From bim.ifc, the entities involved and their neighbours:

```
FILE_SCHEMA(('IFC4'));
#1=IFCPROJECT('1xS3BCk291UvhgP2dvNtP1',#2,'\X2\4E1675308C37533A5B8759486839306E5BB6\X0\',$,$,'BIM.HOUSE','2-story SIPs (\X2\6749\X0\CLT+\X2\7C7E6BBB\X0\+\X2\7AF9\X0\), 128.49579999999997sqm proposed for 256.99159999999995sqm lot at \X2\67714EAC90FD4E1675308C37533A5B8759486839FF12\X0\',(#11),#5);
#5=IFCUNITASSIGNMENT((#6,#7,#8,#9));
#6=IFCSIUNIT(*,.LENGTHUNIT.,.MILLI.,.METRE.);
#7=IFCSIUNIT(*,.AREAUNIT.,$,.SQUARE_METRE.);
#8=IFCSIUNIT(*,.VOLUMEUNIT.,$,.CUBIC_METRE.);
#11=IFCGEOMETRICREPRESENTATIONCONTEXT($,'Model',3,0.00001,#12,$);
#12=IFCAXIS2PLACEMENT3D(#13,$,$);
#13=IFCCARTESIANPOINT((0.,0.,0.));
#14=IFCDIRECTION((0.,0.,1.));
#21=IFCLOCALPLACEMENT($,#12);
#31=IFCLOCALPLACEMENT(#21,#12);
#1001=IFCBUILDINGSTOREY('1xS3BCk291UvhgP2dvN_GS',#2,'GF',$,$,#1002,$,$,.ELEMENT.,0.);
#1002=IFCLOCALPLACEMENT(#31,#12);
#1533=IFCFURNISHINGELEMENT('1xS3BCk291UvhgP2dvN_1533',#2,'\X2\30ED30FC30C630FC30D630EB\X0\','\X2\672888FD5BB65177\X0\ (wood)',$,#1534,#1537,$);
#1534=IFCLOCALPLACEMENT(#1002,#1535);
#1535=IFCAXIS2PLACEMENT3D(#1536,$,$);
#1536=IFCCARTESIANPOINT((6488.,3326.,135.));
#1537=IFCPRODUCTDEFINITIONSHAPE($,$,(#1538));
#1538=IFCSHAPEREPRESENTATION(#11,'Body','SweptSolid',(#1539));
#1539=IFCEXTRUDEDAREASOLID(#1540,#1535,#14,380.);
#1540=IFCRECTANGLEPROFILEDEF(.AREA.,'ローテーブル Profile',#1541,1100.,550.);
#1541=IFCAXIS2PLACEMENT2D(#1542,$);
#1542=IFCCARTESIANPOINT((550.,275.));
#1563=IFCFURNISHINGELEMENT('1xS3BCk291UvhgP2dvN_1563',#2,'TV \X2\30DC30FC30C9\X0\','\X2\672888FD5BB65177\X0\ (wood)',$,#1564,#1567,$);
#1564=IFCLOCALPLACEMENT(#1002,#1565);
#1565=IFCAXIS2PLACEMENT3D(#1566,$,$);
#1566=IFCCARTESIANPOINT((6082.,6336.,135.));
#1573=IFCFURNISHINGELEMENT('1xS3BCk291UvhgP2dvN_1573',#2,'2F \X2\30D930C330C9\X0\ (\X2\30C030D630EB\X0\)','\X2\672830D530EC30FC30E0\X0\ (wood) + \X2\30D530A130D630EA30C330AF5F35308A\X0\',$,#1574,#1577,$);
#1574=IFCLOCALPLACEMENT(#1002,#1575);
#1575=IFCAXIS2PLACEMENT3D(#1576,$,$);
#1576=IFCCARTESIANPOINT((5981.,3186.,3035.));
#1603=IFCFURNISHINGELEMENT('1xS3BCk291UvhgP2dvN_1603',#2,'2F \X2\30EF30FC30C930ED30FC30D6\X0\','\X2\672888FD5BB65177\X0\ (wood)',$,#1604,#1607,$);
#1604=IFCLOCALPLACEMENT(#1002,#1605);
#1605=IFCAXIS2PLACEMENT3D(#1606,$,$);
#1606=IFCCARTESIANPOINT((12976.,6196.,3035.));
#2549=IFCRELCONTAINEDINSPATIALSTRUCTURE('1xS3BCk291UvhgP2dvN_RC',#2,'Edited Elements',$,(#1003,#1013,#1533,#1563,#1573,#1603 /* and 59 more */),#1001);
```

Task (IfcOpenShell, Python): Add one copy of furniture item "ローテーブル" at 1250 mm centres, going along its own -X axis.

```python
import ifcopenshell
import ifcopenshell.api.geometry
import ifcopenshell.api.root
import ifcopenshell.util.element
import ifcopenshell.util.placement
import ifcopenshell.util.unit

model = ifcopenshell.open("bim.ifc")
unit_scale = ifcopenshell.util.unit.calculate_unit_scale(model)


def reuse_history(source, copy):
    """copy_class also copies each property set's owner history, people and application; keep the originals."""
    for rel in copy.IsDefinedBy:
        if rel.is_a("IfcRelDefinesByProperties") and (history := rel.RelatingPropertyDefinition.OwnerHistory):
            rel.RelatingPropertyDefinition.OwnerHistory = source.OwnerHistory
            ifcopenshell.util.element.remove_deep2(model, history)


source = model.by_id(1533)
base = ifcopenshell.util.placement.get_local_placement(source.ObjectPlacement)
step = -base[:3, 0] * 1.25 / unit_scale

for i in range(1, 2):
    copy = ifcopenshell.api.root.copy_class(model, product=source)
    copy.Representation = ifcopenshell.util.element.copy_deep(
        model, source.Representation, exclude=["IfcGeometricRepresentationContext", "IfcRepresentationMap"]
    )
    reuse_history(source, copy)
    matrix = base.copy()
    matrix[:3, 3] += i * step
    print("added at", matrix[:3, 3].round(3) + 0.0)
    ifcopenshell.api.geometry.edit_object_placement(model, product=copy, matrix=matrix, is_si=False)

model.write("bim_rev.ifc")
```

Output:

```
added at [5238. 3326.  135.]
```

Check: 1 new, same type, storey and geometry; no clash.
